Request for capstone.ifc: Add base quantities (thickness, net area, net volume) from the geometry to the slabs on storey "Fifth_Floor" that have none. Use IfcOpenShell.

First a look at what the model holds.

```python
import ifcopenshell
import ifcopenshell.util.element
import ifcopenshell.util.unit

model = ifcopenshell.open("capstone.ifc")
print(model.schema)
for unit_type in ("LENGTHUNIT", "AREAUNIT", "VOLUMEUNIT"):
    print(unit_type, ifcopenshell.util.unit.calculate_unit_scale(model, unit_type))
storey = next(s for s in model.by_type("IfcBuildingStorey") if s.Name == "Fifth_Floor")
slabs = [e for e in ifcopenshell.util.element.get_decomposition(storey) if e.is_a("IfcSlab")]
for e in sorted(slabs, key=lambda e: e.id()):
    print(e.id(), e.is_a(), e.Name, list(ifcopenshell.util.element.get_psets(e, qtos_only=True)), sep=" | ")
```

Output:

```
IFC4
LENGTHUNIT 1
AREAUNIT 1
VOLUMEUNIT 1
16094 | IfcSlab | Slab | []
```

```python
import ifcopenshell
import ifcopenshell.api.pset
import ifcopenshell.geom
import ifcopenshell.util.element
import ifcopenshell.util.shape
import ifcopenshell.util.unit

model = ifcopenshell.open("capstone.ifc")
unit_scale = ifcopenshell.util.unit.calculate_unit_scale(model)
area_scale = ifcopenshell.util.unit.calculate_unit_scale(model, "AREAUNIT")
volume_scale = ifcopenshell.util.unit.calculate_unit_scale(model, "VOLUMEUNIT")
settings = ifcopenshell.geom.settings()

storey = next(s for s in model.by_type("IfcBuildingStorey") if s.Name == "Fifth_Floor")
slabs = [e for e in ifcopenshell.util.element.get_decomposition(storey) if e.is_a("IfcSlab")]

for e in sorted(slabs, key=lambda e: e.id()):
    if ifcopenshell.util.element.get_psets(e, qtos_only=True, should_inherit=False):
        continue
    # Geometry comes back in metres, in the element's own axes.
    shape = ifcopenshell.geom.create_shape(settings, e)
    values = {
        "Width": ifcopenshell.util.shape.get_z(shape.geometry) / unit_scale,
        "NetArea": ifcopenshell.util.shape.get_footprint_area(shape.geometry) / area_scale,
        "NetVolume": ifcopenshell.util.shape.get_volume(shape.geometry) / volume_scale,
    }
    qto = ifcopenshell.api.pset.add_qto(model, product=e, name="Qto_SlabBaseQuantities")
    ifcopenshell.api.pset.edit_qto(model, qto=qto, properties=values)
    print(e.id(), {k: round(v, 3) for k, v in values.items()})

model.write("capstone_v2.ifc")
```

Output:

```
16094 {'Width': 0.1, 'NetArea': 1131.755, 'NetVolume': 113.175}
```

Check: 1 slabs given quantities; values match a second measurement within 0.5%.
